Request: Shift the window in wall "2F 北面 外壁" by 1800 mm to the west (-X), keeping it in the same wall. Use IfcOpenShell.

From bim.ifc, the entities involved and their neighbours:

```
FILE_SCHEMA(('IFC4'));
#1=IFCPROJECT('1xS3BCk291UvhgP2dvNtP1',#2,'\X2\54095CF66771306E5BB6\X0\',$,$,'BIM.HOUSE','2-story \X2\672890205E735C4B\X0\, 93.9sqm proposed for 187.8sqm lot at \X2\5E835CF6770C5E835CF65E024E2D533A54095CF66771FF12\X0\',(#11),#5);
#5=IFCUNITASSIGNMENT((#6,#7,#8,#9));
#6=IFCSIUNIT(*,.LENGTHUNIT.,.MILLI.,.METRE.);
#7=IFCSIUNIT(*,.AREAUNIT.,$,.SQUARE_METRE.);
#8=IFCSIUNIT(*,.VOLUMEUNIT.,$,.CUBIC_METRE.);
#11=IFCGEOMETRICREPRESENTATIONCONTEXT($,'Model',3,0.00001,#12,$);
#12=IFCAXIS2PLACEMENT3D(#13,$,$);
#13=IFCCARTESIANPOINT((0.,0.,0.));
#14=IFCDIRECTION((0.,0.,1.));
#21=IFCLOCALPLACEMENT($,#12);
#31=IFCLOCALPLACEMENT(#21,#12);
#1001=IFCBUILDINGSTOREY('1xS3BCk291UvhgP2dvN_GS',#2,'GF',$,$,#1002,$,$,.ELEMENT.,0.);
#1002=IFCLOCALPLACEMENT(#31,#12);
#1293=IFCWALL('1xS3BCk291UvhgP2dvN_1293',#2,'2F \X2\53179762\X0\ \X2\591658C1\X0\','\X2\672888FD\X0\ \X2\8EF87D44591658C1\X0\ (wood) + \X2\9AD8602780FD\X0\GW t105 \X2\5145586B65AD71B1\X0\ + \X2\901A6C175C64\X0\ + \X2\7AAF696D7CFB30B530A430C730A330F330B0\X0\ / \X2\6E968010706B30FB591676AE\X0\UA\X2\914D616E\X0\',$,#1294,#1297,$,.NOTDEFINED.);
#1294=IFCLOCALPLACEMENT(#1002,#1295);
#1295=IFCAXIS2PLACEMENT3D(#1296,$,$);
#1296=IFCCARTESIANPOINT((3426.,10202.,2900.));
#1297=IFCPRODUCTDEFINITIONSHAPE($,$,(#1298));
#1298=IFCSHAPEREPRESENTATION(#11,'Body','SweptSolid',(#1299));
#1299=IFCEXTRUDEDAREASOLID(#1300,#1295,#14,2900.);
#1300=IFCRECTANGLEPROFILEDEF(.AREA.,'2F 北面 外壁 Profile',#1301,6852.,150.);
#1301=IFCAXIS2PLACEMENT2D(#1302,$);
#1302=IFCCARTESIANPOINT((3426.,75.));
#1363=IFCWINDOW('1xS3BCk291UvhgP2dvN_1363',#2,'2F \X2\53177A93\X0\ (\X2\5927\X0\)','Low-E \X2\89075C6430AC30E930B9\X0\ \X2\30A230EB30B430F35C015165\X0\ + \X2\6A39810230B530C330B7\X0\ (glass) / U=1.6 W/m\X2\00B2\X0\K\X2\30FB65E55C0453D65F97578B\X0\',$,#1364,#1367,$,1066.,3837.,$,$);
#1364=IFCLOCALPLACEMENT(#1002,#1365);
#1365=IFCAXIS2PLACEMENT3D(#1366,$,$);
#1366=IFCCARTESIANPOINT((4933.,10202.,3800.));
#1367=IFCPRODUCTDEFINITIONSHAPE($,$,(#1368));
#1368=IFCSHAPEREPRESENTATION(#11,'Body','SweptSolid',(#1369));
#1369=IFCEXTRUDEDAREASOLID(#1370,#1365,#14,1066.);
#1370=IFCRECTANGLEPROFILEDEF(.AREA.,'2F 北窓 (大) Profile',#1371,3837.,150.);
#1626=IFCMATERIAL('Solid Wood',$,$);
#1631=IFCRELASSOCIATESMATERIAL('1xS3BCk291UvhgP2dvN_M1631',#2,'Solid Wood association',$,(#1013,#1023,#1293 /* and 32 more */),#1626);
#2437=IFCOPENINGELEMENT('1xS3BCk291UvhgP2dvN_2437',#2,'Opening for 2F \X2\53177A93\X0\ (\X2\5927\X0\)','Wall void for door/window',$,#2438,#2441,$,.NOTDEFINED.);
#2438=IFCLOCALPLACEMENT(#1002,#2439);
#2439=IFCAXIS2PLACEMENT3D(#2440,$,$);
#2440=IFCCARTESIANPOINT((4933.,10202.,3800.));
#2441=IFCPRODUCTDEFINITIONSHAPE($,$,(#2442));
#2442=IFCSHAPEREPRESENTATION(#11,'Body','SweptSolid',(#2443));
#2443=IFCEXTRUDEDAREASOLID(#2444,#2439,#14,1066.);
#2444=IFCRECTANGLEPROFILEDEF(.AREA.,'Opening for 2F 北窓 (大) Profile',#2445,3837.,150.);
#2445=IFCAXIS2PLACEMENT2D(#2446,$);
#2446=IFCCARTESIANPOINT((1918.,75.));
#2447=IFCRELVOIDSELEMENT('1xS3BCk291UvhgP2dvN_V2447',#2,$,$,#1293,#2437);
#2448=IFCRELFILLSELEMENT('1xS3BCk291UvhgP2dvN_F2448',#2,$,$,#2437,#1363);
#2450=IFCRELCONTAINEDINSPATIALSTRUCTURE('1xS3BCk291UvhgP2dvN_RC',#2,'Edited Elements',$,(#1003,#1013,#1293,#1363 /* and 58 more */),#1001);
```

```python
import ifcopenshell
import ifcopenshell.api.geometry
import ifcopenshell.util.placement

model = ifcopenshell.open("bim.ifc")

window = model.by_guid("1xS3BCk291UvhgP2dvN_1363")
opening = window.FillsVoids[0].RelatingOpeningElement
wall = opening.VoidsElements[0].RelatingBuildingElement

wall_matrix = ifcopenshell.util.placement.get_local_placement(wall.ObjectPlacement)
shift = wall_matrix[:3, 0] * -1800.0
before = ifcopenshell.util.placement.get_local_placement(window.ObjectPlacement)[:3, 3].copy()

# The window is not placed relative to its opening, so move both.
for product in (opening, window):
    matrix = ifcopenshell.util.placement.get_local_placement(product.ObjectPlacement)
    matrix[:3, 3] += shift
    ifcopenshell.api.geometry.edit_object_placement(model, product=product, matrix=matrix, is_si=False)

after = ifcopenshell.util.placement.get_local_placement(window.ObjectPlacement)[:3, 3]
print("window moved by", (after - before).round(3) + 0.0)

model.write("bim_edited.ifc")
```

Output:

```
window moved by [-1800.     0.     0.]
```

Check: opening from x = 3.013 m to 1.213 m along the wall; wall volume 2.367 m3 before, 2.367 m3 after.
